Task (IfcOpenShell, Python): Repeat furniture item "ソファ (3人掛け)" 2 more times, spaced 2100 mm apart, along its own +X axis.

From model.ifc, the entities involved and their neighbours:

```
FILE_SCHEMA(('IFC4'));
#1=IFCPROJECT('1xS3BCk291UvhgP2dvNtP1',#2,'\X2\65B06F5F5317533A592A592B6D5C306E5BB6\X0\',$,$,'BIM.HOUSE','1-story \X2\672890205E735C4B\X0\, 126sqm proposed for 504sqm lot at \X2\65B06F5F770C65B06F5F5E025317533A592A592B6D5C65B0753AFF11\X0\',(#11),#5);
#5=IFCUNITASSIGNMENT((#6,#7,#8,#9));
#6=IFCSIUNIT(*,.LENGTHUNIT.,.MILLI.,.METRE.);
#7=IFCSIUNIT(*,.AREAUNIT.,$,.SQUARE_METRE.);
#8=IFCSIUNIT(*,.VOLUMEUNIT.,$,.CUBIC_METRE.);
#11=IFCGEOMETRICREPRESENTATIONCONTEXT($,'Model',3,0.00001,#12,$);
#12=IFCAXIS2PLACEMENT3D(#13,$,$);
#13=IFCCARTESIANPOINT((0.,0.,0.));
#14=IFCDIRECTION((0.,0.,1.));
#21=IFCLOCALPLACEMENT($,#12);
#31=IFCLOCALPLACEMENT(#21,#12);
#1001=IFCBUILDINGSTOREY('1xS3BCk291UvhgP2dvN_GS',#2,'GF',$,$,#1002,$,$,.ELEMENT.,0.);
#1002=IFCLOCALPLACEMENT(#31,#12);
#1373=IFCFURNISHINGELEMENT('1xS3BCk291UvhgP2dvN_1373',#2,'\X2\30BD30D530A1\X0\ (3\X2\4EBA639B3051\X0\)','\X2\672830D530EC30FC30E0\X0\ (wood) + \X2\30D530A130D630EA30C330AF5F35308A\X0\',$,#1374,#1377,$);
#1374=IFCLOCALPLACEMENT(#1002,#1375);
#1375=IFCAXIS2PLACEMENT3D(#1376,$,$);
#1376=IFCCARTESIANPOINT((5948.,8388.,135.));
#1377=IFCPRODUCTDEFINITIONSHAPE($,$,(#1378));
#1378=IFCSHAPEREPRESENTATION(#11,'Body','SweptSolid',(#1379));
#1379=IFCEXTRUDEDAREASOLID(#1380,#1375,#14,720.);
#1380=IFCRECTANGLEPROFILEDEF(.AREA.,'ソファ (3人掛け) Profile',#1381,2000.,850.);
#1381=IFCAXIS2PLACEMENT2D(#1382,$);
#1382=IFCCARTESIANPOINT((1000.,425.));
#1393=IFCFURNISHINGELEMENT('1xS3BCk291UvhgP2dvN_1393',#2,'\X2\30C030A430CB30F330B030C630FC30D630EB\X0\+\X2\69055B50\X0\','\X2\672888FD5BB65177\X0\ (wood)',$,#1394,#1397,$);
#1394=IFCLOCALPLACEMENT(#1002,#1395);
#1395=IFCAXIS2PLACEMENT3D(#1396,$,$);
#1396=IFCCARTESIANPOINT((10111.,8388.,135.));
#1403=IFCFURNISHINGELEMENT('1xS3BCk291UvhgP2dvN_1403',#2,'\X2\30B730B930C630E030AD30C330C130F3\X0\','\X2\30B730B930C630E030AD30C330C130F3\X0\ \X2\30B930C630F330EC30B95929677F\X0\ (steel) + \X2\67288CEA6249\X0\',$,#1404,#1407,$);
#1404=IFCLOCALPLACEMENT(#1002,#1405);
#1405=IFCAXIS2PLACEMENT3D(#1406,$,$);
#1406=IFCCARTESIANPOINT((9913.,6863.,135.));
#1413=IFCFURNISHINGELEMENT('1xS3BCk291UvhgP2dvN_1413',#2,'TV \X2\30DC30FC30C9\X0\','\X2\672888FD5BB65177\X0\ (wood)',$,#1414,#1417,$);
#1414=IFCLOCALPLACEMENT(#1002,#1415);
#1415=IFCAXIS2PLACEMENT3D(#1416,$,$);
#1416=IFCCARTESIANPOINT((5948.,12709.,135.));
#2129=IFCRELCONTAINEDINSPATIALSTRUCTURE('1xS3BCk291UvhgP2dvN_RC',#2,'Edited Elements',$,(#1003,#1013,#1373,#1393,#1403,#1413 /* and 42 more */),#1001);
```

```python
import ifcopenshell
import ifcopenshell.api.geometry
import ifcopenshell.api.root
import ifcopenshell.util.element
import ifcopenshell.util.placement
import ifcopenshell.util.unit

model = ifcopenshell.open("model.ifc")
unit_scale = ifcopenshell.util.unit.calculate_unit_scale(model)


def reuse_history(source, copy):
    """copy_class also copies each property set's owner history, people and application; keep the originals."""
    for rel in copy.IsDefinedBy:
        if rel.is_a("IfcRelDefinesByProperties") and (history := rel.RelatingPropertyDefinition.OwnerHistory):
            rel.RelatingPropertyDefinition.OwnerHistory = source.OwnerHistory
            ifcopenshell.util.element.remove_deep2(model, history)


source = model.by_guid("1xS3BCk291UvhgP2dvN_1373")
base = ifcopenshell.util.placement.get_local_placement(source.ObjectPlacement)
step = base[:3, 0] * 2.1 / unit_scale

for i in range(1, 3):
    copy = ifcopenshell.api.root.copy_class(model, product=source)
    copy.Representation = ifcopenshell.util.element.copy_deep(
        model, source.Representation, exclude=["IfcGeometricRepresentationContext", "IfcRepresentationMap"]
    )
    reuse_history(source, copy)
    matrix = base.copy()
    matrix[:3, 3] += i * step
    print("added at", matrix[:3, 3].round(3) + 0.0)
    ifcopenshell.api.geometry.edit_object_placement(model, product=copy, matrix=matrix, is_si=False)

model.write("model_rev.ifc")
```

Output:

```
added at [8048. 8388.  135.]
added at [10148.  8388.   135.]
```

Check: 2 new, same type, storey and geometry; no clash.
